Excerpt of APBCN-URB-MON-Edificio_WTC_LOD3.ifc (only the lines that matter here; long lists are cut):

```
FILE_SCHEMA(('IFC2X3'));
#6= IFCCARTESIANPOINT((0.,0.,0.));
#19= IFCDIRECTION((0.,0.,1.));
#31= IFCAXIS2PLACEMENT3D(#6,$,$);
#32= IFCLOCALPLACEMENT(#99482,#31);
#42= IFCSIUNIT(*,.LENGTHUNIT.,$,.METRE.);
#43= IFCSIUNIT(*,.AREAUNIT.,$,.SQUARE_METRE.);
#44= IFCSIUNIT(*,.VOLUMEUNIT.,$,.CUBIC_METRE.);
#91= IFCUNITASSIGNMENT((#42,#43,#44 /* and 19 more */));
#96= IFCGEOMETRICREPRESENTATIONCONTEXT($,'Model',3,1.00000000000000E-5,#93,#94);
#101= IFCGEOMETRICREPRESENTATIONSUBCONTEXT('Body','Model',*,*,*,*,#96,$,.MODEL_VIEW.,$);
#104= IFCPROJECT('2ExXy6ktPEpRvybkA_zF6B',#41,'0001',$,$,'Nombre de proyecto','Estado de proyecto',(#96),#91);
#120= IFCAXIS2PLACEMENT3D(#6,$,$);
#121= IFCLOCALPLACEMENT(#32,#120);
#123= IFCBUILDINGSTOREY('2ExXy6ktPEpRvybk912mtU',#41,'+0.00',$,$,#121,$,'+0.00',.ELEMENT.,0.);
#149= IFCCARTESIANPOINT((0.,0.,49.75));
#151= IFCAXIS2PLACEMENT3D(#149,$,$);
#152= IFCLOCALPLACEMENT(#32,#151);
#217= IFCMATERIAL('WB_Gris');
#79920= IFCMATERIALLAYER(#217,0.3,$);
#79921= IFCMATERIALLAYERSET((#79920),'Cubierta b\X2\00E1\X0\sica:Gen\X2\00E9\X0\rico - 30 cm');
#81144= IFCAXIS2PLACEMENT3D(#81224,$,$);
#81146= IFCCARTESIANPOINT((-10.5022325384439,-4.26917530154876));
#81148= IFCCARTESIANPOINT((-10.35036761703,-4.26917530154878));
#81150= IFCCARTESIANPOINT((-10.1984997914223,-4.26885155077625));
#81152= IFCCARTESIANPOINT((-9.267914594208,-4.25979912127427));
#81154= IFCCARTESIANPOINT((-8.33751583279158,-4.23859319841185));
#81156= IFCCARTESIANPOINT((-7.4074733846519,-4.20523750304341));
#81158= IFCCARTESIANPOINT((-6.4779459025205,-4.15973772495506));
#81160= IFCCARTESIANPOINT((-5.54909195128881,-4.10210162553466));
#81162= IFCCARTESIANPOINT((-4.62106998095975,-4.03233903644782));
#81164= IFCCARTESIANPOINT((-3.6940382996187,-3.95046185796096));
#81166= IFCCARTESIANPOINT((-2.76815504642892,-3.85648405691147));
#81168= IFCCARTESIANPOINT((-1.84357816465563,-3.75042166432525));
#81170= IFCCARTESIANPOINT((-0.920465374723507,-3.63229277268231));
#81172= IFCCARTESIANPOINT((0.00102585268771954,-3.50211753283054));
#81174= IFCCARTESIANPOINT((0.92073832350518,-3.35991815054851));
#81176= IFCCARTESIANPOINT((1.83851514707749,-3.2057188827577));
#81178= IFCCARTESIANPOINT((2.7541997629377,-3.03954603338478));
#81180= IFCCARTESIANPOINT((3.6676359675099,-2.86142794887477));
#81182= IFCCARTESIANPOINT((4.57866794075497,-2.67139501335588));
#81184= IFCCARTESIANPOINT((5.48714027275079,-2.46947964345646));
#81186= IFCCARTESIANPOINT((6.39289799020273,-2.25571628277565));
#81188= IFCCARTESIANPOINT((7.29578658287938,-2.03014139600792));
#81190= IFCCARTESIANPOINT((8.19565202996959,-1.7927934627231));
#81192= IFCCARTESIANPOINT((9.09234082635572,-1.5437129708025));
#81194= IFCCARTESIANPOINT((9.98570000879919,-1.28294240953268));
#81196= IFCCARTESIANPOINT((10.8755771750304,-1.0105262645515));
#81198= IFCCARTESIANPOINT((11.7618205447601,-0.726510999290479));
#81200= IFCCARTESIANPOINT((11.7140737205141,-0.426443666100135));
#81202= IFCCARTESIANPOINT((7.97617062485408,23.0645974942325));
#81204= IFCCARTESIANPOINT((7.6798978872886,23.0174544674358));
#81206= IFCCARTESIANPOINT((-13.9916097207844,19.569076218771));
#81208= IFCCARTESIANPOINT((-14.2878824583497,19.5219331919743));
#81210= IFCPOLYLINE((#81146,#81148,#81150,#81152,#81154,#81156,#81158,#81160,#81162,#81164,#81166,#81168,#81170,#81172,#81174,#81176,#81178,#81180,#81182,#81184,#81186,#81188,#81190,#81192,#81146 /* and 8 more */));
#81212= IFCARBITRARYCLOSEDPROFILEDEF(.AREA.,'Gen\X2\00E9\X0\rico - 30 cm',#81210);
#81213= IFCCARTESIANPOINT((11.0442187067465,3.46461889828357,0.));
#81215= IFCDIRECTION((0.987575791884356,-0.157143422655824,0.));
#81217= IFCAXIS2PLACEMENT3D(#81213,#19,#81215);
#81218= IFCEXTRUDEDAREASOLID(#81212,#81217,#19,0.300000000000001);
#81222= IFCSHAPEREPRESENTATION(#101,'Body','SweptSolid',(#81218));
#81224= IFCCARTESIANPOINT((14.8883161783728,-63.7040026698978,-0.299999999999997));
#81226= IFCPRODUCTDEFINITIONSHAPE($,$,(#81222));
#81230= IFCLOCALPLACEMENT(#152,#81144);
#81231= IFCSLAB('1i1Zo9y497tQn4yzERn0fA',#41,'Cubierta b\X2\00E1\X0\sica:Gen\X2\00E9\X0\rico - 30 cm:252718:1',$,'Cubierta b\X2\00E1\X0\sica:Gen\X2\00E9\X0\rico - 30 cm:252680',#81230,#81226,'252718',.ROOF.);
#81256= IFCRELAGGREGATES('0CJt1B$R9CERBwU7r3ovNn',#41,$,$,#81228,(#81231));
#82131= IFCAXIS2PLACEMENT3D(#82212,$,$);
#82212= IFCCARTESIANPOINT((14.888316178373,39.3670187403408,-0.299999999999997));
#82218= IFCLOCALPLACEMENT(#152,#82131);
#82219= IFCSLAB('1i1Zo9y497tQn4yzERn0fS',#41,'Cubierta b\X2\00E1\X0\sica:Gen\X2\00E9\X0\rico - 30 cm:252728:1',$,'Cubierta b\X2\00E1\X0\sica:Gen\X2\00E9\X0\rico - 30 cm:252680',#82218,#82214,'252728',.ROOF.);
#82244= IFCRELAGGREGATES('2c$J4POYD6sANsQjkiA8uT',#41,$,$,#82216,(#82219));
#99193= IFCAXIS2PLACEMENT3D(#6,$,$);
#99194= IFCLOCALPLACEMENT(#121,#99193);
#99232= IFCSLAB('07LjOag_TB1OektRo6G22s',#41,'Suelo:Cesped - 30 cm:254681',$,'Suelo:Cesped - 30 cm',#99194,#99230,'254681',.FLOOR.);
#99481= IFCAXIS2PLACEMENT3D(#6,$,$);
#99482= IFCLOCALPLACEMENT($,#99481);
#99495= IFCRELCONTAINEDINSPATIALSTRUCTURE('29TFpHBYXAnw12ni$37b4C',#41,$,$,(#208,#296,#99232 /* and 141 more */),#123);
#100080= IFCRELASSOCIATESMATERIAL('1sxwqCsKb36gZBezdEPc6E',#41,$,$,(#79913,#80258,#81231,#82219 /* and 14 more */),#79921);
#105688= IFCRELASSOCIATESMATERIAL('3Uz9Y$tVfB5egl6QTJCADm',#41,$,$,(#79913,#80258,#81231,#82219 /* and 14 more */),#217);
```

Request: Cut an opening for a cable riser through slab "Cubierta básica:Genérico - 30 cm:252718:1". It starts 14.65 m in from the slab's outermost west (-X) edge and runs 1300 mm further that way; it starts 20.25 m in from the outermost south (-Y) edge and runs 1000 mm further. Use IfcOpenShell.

```python
import numpy as np
import ifcopenshell
import ifcopenshell.api.feature
import ifcopenshell.api.geometry
import ifcopenshell.api.root
import ifcopenshell.geom
import ifcopenshell.util.placement
import ifcopenshell.util.representation
import ifcopenshell.util.shape
import ifcopenshell.util.unit

model = ifcopenshell.open("APBCN-URB-MON-Edificio_WTC_LOD3.ifc")
unit_scale = ifcopenshell.util.unit.calculate_unit_scale(model)
settings = ifcopenshell.geom.settings()


def volume(element):
    """Net volume in cubic metres, openings subtracted."""
    shape = ifcopenshell.geom.create_shape(settings, element)
    return ifcopenshell.util.shape.get_volume(shape.geometry)


slab = model.by_id(81231)
before = volume(slab)

# Extent in the slab's own axes, in metres. The edges named are its -X and -Y sides.
slab_shape = ifcopenshell.geom.create_shape(settings, slab)
vertices = ifcopenshell.util.shape.get_vertices(slab_shape.geometry)
x_min, y_min, bottom = vertices.min(axis=0)
top = vertices[:, 2].max()

opening = ifcopenshell.api.root.create_entity(model, ifc_class="IfcOpeningElement", name="Cable riser opening")
context = ifcopenshell.util.representation.get_context(model, "Model", "Body", "MODEL_VIEW")
width, depth = 1.3, 1
outline = [(0.0, 0.0), (width, 0.0), (width, depth), (0.0, depth), (0.0, 0.0)]
# Overshoot both faces by 50 mm so the cut is clean.
shape = ifcopenshell.api.geometry.add_slab_representation(
    model, context=context, depth=top - bottom + 0.1, polyline=outline
)
ifcopenshell.api.geometry.assign_representation(model, product=opening, representation=shape)

matrix = ifcopenshell.util.placement.get_local_placement(slab.ObjectPlacement)
matrix[:, 3] = matrix @ np.append(np.array([x_min + 14.65, y_min + 20.25, bottom - 0.05]) / unit_scale, 1.0)
ifcopenshell.api.geometry.edit_object_placement(model, product=opening, matrix=matrix, is_si=False)
ifcopenshell.api.feature.add_feature(model, feature=opening, element=slab)

after = volume(slab)

print(f"slab volume {before:.3f} -> {after:.3f} m3")

model.write("APBCN-URB-MON-Edificio_WTC_LOD3_updated.ifc")
```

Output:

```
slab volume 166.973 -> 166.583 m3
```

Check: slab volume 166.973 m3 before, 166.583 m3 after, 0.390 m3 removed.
